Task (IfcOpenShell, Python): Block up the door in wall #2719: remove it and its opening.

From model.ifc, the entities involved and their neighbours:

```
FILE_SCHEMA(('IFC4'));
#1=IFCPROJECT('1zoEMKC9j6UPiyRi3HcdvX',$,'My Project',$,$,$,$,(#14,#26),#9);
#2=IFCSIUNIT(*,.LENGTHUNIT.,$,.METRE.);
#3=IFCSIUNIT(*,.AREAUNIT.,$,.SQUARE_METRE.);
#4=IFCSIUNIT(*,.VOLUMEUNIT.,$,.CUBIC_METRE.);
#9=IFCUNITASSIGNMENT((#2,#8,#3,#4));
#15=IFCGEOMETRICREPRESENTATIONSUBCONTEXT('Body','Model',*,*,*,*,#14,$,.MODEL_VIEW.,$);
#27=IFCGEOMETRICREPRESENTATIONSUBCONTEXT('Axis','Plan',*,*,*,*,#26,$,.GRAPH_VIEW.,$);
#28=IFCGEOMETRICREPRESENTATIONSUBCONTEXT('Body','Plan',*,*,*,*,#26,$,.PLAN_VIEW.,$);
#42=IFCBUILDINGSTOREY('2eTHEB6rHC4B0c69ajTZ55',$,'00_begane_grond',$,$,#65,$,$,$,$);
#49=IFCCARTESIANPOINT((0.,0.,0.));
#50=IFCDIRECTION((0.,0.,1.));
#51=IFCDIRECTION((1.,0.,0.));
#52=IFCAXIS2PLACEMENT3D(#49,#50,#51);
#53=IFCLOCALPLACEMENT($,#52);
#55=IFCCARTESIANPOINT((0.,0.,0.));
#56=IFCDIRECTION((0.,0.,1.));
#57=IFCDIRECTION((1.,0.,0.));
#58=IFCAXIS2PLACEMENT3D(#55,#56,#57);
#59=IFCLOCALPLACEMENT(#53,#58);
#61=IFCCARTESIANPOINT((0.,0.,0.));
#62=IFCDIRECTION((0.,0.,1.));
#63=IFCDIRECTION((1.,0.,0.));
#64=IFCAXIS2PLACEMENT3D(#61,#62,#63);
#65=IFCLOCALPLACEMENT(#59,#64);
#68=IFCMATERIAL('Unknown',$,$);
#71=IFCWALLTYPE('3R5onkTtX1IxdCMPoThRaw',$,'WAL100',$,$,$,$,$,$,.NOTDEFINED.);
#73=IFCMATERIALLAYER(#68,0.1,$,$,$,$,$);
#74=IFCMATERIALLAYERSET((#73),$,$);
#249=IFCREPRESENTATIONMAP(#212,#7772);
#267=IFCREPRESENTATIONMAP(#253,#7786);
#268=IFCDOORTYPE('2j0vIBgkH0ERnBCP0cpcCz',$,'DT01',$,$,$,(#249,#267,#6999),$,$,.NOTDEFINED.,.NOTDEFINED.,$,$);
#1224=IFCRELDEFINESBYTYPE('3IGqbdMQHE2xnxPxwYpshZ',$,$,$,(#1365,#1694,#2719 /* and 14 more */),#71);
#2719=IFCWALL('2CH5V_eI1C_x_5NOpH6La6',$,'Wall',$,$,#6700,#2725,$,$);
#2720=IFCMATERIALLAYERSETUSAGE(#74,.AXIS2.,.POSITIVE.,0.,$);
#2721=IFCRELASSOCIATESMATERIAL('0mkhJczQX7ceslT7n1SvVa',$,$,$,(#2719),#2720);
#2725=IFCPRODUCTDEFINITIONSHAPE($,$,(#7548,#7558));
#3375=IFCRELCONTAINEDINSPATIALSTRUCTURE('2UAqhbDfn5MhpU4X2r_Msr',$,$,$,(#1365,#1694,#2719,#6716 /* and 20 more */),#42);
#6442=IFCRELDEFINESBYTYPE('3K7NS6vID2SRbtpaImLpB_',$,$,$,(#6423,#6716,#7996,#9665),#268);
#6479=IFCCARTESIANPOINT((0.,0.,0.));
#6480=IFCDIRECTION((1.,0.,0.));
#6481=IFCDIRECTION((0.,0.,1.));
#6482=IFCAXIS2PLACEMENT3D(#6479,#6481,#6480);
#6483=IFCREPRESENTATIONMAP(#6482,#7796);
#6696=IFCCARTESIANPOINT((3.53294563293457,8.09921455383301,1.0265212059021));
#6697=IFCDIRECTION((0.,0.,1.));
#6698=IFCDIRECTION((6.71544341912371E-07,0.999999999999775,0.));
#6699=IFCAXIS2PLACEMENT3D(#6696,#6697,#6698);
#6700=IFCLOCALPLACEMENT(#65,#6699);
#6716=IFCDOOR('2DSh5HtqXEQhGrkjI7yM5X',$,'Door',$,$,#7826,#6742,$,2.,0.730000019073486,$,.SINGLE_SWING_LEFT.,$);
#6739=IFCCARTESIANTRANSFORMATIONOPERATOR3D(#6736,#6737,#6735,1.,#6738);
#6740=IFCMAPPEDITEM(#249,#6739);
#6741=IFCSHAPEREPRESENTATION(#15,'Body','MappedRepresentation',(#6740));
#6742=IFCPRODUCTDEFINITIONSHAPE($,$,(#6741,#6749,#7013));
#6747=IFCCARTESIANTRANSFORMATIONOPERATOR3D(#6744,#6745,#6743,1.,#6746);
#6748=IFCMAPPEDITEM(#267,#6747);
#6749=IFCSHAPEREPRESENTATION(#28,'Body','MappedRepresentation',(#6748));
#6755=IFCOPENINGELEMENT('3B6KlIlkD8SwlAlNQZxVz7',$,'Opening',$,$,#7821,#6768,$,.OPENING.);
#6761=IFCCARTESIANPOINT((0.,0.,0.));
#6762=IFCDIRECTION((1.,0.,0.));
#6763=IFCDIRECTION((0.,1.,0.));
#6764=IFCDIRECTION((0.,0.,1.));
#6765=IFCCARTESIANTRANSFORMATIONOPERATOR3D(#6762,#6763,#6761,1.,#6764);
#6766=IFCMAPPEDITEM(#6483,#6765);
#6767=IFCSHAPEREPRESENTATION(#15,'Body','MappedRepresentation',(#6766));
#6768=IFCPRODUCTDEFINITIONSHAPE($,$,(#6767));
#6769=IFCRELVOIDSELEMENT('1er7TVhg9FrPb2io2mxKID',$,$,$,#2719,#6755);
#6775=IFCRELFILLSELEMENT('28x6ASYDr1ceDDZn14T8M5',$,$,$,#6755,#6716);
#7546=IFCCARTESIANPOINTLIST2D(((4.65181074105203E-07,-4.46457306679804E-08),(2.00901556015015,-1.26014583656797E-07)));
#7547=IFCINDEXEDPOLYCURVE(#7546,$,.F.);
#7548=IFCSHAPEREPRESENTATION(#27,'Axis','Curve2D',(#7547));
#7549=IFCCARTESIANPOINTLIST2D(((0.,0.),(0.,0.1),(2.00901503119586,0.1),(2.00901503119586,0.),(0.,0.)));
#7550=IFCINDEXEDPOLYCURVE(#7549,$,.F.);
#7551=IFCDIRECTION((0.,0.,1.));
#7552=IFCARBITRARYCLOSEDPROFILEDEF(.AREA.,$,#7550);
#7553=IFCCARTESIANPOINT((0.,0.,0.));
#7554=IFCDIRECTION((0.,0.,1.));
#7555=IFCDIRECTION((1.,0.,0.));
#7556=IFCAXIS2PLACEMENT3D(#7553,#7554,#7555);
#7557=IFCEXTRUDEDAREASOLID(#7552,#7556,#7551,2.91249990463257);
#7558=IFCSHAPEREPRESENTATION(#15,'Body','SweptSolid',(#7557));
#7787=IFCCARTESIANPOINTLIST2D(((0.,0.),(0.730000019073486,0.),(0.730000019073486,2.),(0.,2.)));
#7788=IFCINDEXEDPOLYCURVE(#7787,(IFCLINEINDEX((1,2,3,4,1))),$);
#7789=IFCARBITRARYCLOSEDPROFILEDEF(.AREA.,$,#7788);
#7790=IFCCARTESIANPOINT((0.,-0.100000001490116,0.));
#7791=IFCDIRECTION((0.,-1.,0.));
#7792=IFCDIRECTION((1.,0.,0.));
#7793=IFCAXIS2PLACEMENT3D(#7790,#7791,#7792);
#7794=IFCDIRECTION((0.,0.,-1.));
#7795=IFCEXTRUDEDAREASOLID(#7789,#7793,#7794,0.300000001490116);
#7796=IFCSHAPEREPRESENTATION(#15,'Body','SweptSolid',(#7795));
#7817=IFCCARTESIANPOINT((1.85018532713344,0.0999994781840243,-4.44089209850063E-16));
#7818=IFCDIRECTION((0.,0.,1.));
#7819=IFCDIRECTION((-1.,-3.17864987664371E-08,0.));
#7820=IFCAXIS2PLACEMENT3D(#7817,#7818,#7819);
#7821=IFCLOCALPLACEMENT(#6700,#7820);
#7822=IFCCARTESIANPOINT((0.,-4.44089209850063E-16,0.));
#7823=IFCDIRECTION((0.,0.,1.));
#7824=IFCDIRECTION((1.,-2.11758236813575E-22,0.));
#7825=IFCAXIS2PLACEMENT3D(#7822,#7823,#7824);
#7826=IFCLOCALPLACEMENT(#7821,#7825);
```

```python
import ifcopenshell
import ifcopenshell.api.feature
import ifcopenshell.api.root
import ifcopenshell.geom
import ifcopenshell.util.shape

model = ifcopenshell.open("model.ifc")
settings = ifcopenshell.geom.settings()


def volume(element):
    """Net volume in cubic metres, openings subtracted."""
    shape = ifcopenshell.geom.create_shape(settings, element)
    return ifcopenshell.util.shape.get_volume(shape.geometry)


door = model.by_guid("2DSh5HtqXEQhGrkjI7yM5X")
opening = door.FillsVoids[0].RelatingOpeningElement
wall = opening.VoidsElements[0].RelatingBuildingElement
before = volume(wall)

ifcopenshell.api.root.remove_product(model, product=door)
ifcopenshell.api.feature.remove_feature(model, feature=opening)

after = volume(wall)

print(f"wall volume {before:.3f} -> {after:.3f} m3")

model.write("model_updated.ifc")
```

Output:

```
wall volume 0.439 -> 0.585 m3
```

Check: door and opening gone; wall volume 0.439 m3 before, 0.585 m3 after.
